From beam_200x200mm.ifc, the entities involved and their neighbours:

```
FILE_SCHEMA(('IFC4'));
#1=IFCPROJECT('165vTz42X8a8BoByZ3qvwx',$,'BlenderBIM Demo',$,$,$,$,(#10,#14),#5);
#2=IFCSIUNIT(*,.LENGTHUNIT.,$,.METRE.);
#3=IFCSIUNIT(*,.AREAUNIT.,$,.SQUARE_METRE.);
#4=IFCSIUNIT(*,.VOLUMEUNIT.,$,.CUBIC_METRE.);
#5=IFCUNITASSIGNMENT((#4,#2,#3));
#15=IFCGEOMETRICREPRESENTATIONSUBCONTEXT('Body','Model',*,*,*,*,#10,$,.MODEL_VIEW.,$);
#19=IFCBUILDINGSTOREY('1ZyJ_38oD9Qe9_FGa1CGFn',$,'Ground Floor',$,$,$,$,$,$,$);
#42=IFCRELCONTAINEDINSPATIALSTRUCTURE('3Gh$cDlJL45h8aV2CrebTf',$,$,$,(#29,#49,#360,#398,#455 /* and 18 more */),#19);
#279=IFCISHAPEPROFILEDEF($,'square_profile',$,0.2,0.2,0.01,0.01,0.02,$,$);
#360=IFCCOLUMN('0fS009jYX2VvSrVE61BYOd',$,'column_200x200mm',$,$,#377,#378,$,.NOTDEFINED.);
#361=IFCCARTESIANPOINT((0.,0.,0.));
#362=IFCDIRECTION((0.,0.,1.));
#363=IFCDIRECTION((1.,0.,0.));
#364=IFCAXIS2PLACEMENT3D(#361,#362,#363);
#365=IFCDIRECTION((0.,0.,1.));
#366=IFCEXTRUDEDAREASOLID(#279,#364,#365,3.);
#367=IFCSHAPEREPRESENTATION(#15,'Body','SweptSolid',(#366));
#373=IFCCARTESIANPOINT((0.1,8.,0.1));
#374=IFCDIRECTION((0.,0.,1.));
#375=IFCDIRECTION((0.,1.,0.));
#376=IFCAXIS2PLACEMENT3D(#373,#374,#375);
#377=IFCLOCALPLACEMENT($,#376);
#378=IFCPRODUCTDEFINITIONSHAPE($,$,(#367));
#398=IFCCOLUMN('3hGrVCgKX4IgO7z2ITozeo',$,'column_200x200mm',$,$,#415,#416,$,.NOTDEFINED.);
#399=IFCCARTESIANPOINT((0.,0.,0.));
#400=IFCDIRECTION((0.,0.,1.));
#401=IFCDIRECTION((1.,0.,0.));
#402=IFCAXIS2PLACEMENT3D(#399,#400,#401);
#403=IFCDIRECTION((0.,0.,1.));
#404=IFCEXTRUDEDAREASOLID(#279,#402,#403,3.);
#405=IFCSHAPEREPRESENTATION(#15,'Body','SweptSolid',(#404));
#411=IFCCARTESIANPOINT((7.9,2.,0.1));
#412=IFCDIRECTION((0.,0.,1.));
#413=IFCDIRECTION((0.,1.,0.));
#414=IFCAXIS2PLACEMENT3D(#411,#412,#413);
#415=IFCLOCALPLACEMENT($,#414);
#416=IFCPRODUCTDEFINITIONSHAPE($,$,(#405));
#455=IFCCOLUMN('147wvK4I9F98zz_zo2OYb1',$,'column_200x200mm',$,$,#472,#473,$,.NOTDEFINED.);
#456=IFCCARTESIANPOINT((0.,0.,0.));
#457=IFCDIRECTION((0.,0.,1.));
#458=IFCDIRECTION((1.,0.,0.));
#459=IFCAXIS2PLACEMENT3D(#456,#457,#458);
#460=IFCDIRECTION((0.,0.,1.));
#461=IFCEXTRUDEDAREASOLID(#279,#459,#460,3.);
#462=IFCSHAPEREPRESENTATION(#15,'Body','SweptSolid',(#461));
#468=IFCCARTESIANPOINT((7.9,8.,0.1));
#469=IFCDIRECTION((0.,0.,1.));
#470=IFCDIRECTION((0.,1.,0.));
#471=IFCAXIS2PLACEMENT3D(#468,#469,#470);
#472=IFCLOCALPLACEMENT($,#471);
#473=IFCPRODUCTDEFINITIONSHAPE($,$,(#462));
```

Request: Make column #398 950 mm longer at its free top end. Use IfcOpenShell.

```python
import ifcopenshell
import ifcopenshell.util.representation
import ifcopenshell.util.unit

model = ifcopenshell.open("beam_200x200mm.ifc")
unit_scale = ifcopenshell.util.unit.calculate_unit_scale(model)

member = model.by_id(398)
change = 0.95 / unit_scale

# The extrusion runs towards the end named, so only its depth changes.
body = ifcopenshell.util.representation.get_representation(member, "Model", "Body")
solid = body.Items[0]
old_length = solid.Depth
solid.Depth += change

print(f"length {old_length:g} -> {solid.Depth:g}")

model.write("beam_200x200mm-out.ifc")
```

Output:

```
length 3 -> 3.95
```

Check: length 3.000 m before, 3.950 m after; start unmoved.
